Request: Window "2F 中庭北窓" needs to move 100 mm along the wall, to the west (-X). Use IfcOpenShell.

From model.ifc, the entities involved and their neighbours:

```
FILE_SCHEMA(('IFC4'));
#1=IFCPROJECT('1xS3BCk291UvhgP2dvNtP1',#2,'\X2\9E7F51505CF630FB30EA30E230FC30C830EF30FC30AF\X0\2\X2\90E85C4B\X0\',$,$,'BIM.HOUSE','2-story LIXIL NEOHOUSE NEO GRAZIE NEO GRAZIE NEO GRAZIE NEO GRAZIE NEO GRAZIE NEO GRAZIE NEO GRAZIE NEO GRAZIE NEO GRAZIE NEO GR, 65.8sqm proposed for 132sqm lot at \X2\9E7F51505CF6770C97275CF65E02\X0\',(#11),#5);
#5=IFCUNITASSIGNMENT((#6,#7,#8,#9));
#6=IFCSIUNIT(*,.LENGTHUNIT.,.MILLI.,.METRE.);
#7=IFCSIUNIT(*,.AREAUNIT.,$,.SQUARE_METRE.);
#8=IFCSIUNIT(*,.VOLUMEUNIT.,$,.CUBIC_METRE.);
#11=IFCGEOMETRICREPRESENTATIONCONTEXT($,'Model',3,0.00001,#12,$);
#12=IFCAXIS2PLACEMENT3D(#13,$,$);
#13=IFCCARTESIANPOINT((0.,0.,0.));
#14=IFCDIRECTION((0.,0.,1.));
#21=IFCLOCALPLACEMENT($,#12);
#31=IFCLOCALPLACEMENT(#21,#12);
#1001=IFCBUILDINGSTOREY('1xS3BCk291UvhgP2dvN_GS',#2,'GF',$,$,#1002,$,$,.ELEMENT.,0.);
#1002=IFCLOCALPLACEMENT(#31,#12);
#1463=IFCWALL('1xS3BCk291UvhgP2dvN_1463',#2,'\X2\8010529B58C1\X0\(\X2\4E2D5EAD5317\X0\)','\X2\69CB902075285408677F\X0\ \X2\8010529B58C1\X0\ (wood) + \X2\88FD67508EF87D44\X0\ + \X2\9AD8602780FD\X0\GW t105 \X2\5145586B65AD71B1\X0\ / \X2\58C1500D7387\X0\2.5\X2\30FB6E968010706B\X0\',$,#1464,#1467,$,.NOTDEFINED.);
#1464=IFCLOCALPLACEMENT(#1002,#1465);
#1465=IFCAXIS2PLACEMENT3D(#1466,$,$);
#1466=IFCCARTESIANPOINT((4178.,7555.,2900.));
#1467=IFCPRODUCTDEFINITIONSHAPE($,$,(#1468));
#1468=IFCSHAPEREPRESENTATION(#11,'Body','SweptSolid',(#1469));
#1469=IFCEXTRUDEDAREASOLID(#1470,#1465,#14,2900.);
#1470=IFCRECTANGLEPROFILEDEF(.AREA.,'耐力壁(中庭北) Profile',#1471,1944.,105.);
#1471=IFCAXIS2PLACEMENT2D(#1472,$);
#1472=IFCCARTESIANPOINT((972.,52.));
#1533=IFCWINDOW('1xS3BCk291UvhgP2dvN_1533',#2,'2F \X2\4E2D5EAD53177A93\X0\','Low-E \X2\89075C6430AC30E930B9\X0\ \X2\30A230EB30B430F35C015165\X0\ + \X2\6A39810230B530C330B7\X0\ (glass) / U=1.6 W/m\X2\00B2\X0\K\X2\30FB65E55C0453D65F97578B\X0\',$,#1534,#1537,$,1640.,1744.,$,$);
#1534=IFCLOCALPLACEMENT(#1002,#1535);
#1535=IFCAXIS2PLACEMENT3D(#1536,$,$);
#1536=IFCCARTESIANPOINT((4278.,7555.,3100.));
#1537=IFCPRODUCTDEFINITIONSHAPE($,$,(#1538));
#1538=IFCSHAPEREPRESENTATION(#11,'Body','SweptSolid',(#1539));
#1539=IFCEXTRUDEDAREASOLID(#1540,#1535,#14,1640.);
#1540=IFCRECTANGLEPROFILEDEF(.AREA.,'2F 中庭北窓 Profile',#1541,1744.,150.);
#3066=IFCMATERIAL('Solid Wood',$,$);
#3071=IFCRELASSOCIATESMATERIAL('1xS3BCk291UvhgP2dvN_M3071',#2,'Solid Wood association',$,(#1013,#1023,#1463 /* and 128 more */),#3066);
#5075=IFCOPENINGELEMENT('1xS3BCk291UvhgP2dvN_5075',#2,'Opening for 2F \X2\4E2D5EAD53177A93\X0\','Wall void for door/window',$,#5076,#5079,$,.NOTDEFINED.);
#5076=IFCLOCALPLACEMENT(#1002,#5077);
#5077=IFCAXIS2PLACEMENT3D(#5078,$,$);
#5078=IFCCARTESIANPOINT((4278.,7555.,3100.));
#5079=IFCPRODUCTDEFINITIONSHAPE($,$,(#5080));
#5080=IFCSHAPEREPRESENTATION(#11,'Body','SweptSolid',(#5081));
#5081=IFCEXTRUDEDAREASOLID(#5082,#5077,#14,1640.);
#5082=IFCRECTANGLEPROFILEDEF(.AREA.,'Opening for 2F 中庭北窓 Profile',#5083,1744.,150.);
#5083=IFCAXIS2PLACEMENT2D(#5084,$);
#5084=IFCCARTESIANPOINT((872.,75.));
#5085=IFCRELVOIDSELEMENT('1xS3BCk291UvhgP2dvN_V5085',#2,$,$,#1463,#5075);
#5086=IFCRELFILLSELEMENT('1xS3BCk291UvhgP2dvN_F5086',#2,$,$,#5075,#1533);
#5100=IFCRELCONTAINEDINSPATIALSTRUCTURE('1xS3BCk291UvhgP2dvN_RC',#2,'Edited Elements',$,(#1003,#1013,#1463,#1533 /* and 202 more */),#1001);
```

```python
import ifcopenshell
import ifcopenshell.api.geometry
import ifcopenshell.util.placement

model = ifcopenshell.open("model.ifc")

window = model.by_guid("1xS3BCk291UvhgP2dvN_1533")
opening = window.FillsVoids[0].RelatingOpeningElement
wall = opening.VoidsElements[0].RelatingBuildingElement

wall_matrix = ifcopenshell.util.placement.get_local_placement(wall.ObjectPlacement)
shift = wall_matrix[:3, 0] * -100.0
before = ifcopenshell.util.placement.get_local_placement(window.ObjectPlacement)[:3, 3].copy()

# The window is not placed relative to its opening, so move both.
for product in (opening, window):
    matrix = ifcopenshell.util.placement.get_local_placement(product.ObjectPlacement)
    matrix[:3, 3] += shift
    ifcopenshell.api.geometry.edit_object_placement(model, product=product, matrix=matrix, is_si=False)

after = ifcopenshell.util.placement.get_local_placement(window.ObjectPlacement)[:3, 3]
print("window moved by", (after - before).round(3) + 0.0)

model.write("model_v2.ifc")
```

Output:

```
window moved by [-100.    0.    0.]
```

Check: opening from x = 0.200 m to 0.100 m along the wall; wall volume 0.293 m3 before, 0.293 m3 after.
